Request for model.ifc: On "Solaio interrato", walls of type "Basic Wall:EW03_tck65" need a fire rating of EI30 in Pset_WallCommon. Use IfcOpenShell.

First a look at what the model holds.

```python
import ifcopenshell
import ifcopenshell.util.element

model = ifcopenshell.open("model.ifc")
print(model.schema)
storey = next(s for s in model.by_type("IfcBuildingStorey") if s.Name == "Solaio interrato")
walls = [e for e in ifcopenshell.util.element.get_decomposition(storey) if e.is_a("IfcWall")]
seen = {}
for e in walls:
    element_type = ifcopenshell.util.element.get_type(e)
    key = (element_type.Name if element_type != e and element_type else None, ifcopenshell.util.element.get_pset(e, "Pset_WallCommon", "FireRating"))
    seen[key] = seen.get(key, 0) + 1
for (name, value), count in sorted(seen.items(), key=str):
    print(count, "x", name, "|", value)
```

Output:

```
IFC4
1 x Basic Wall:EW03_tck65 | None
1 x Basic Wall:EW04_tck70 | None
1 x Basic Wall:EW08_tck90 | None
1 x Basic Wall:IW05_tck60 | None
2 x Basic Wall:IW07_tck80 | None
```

```python
import ifcopenshell
import ifcopenshell.api.pset
import ifcopenshell.util.element

model = ifcopenshell.open("model.ifc")

storey = next(s for s in model.by_type("IfcBuildingStorey") if s.Name == "Solaio interrato")
walls = [e for e in ifcopenshell.util.element.get_decomposition(storey) if e.is_a("IfcWall")]

count = 0
for e in walls:
    element_type = ifcopenshell.util.element.get_type(e)
    if element_type in (None, e) or element_type.Name != "Basic Wall:EW03_tck65":
        continue
    found = ifcopenshell.util.element.get_pset(e, "Pset_WallCommon", should_inherit=False)
    if found:
        pset = model.by_id(found["id"])
        if len(ifcopenshell.util.element.get_elements_by_pset(pset)) > 1:
            pset = ifcopenshell.api.pset.unshare_pset(model, products=[e], pset=pset)[0]
    else:
        pset = ifcopenshell.api.pset.add_pset(model, product=e, name="Pset_WallCommon")
    ifcopenshell.api.pset.edit_pset(model, pset=pset, properties={"FireRating": "EI30"})
    count += 1

print(count, "walls updated")

model.write("model_updated.ifc")
```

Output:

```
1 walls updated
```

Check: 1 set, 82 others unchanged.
